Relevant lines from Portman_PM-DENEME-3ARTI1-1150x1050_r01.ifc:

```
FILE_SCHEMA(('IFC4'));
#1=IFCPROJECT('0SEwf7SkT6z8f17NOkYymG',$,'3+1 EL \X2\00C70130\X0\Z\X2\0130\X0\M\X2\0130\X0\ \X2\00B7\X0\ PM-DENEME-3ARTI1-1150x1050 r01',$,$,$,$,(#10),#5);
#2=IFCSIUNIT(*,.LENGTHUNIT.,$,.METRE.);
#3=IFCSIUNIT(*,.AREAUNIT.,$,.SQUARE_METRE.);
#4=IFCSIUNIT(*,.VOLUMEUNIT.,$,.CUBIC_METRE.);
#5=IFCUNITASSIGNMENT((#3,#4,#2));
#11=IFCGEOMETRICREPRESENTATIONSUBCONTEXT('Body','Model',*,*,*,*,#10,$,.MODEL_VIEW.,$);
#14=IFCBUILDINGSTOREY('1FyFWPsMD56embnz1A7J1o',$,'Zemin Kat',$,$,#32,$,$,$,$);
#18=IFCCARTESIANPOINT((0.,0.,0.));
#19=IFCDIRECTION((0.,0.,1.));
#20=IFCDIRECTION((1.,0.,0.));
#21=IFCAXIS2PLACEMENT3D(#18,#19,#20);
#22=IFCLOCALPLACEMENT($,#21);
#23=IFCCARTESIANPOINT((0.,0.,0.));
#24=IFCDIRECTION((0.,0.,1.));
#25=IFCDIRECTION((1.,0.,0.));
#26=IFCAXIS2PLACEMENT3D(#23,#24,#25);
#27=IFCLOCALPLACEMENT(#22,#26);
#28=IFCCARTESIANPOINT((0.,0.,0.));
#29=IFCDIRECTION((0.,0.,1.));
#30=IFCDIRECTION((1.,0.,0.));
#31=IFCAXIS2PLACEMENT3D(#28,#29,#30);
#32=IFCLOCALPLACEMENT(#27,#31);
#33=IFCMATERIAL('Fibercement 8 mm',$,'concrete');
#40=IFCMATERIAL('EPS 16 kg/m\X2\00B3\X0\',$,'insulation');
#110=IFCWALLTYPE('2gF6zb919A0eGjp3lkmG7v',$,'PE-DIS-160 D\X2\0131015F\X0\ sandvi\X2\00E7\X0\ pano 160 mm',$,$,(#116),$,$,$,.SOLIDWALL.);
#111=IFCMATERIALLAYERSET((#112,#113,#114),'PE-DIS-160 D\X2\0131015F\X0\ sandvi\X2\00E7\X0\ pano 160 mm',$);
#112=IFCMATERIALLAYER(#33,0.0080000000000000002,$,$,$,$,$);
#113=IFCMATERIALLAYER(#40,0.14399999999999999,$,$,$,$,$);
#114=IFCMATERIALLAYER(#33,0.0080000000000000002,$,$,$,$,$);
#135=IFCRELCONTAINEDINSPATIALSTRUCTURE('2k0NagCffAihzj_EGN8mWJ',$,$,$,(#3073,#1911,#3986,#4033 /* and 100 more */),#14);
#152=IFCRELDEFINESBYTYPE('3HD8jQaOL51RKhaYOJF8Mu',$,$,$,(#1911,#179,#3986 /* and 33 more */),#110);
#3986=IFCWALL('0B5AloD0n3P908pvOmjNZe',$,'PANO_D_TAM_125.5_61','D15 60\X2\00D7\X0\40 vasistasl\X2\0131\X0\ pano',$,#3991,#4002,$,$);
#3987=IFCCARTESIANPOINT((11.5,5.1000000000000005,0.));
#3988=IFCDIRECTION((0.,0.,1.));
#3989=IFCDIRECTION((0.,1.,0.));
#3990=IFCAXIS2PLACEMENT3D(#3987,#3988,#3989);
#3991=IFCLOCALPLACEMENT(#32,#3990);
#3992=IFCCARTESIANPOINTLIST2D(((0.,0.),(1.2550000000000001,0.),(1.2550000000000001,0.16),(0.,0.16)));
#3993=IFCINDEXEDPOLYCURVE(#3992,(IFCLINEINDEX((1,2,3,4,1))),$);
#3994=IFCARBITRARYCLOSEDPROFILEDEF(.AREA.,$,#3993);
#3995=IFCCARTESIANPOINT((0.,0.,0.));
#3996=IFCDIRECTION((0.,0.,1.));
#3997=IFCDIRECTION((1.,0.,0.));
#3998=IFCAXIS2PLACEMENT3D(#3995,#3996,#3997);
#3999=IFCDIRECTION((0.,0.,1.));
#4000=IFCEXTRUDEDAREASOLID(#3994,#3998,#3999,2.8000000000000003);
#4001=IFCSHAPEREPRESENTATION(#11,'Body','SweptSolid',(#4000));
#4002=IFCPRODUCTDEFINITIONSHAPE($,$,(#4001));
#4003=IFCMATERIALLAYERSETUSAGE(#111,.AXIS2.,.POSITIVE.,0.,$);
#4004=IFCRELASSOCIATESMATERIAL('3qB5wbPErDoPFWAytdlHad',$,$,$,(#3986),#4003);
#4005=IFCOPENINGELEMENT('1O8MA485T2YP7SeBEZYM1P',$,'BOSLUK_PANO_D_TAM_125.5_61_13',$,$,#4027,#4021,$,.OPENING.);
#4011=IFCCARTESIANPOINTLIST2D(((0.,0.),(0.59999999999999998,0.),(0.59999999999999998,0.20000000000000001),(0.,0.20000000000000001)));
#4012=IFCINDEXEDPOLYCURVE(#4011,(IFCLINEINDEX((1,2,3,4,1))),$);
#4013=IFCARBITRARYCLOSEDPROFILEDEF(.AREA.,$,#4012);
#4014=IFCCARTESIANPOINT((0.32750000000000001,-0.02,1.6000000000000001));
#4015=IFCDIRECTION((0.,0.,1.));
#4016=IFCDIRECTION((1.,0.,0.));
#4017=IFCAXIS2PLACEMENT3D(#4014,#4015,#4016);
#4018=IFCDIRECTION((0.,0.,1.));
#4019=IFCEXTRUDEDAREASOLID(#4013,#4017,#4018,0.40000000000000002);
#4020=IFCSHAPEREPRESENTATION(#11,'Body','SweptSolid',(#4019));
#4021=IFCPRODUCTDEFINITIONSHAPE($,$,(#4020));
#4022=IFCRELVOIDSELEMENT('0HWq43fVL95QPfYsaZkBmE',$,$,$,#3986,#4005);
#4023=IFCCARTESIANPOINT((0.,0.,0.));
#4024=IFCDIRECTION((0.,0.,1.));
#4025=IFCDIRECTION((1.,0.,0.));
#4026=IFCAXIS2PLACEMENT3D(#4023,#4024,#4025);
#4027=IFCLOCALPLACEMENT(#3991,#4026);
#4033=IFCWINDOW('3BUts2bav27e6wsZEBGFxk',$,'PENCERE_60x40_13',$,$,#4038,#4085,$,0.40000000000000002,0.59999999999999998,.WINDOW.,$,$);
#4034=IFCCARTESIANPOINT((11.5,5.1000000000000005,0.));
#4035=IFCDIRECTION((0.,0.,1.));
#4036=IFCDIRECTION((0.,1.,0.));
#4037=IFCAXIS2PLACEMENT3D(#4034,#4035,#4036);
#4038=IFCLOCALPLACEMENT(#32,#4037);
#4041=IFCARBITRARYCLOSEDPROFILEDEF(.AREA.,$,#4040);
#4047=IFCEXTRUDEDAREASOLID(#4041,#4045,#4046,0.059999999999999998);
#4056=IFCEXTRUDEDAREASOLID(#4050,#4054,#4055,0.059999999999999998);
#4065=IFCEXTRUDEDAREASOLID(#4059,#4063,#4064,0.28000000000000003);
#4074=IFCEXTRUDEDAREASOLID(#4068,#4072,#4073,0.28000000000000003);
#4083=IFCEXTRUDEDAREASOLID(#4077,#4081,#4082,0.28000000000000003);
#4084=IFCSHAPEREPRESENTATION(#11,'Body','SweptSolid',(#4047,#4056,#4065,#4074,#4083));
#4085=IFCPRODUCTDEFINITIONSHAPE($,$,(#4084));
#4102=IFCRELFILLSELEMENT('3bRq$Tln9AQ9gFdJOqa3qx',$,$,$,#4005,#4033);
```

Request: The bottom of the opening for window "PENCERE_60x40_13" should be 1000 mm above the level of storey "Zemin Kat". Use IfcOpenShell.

```python
import numpy as np
import ifcopenshell
import ifcopenshell.api.geometry
import ifcopenshell.geom
import ifcopenshell.util.element
import ifcopenshell.util.placement
import ifcopenshell.util.shape
import ifcopenshell.util.unit

model = ifcopenshell.open("Portman_PM-DENEME-3ARTI1-1150x1050_r01.ifc")
unit_scale = ifcopenshell.util.unit.calculate_unit_scale(model)

window = model.by_guid("3BUts2bav27e6wsZEBGFxk")
opening = window.FillsVoids[0].RelatingOpeningElement
storey = ifcopenshell.util.element.get_container(window, ifc_class="IfcBuildingStorey")
level = ifcopenshell.util.placement.get_local_placement(storey.ObjectPlacement)[2, 3]

# The opening's origin need not be at the sill, so measure its lowest point.
shape = ifcopenshell.geom.create_shape(ifcopenshell.geom.settings(), opening)
bottom = ifcopenshell.util.shape.get_shape_bottom_elevation(shape, shape.geometry) / unit_scale
dz = level + 1 / unit_scale - bottom

shift = np.array([0.0, 0.0, dz])
# The window is not placed relative to its opening, so move both.
for product in (opening, window):
    matrix = ifcopenshell.util.placement.get_local_placement(product.ObjectPlacement)
    matrix[:3, 3] += shift
    ifcopenshell.api.geometry.edit_object_placement(model, product=product, matrix=matrix, is_si=False)

print(f"moved by {dz * unit_scale:+.3f} m")

model.write("Portman_PM-DENEME-3ARTI1-1150x1050_r01-out.ifc")
```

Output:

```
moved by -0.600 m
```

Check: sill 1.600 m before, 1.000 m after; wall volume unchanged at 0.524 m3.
